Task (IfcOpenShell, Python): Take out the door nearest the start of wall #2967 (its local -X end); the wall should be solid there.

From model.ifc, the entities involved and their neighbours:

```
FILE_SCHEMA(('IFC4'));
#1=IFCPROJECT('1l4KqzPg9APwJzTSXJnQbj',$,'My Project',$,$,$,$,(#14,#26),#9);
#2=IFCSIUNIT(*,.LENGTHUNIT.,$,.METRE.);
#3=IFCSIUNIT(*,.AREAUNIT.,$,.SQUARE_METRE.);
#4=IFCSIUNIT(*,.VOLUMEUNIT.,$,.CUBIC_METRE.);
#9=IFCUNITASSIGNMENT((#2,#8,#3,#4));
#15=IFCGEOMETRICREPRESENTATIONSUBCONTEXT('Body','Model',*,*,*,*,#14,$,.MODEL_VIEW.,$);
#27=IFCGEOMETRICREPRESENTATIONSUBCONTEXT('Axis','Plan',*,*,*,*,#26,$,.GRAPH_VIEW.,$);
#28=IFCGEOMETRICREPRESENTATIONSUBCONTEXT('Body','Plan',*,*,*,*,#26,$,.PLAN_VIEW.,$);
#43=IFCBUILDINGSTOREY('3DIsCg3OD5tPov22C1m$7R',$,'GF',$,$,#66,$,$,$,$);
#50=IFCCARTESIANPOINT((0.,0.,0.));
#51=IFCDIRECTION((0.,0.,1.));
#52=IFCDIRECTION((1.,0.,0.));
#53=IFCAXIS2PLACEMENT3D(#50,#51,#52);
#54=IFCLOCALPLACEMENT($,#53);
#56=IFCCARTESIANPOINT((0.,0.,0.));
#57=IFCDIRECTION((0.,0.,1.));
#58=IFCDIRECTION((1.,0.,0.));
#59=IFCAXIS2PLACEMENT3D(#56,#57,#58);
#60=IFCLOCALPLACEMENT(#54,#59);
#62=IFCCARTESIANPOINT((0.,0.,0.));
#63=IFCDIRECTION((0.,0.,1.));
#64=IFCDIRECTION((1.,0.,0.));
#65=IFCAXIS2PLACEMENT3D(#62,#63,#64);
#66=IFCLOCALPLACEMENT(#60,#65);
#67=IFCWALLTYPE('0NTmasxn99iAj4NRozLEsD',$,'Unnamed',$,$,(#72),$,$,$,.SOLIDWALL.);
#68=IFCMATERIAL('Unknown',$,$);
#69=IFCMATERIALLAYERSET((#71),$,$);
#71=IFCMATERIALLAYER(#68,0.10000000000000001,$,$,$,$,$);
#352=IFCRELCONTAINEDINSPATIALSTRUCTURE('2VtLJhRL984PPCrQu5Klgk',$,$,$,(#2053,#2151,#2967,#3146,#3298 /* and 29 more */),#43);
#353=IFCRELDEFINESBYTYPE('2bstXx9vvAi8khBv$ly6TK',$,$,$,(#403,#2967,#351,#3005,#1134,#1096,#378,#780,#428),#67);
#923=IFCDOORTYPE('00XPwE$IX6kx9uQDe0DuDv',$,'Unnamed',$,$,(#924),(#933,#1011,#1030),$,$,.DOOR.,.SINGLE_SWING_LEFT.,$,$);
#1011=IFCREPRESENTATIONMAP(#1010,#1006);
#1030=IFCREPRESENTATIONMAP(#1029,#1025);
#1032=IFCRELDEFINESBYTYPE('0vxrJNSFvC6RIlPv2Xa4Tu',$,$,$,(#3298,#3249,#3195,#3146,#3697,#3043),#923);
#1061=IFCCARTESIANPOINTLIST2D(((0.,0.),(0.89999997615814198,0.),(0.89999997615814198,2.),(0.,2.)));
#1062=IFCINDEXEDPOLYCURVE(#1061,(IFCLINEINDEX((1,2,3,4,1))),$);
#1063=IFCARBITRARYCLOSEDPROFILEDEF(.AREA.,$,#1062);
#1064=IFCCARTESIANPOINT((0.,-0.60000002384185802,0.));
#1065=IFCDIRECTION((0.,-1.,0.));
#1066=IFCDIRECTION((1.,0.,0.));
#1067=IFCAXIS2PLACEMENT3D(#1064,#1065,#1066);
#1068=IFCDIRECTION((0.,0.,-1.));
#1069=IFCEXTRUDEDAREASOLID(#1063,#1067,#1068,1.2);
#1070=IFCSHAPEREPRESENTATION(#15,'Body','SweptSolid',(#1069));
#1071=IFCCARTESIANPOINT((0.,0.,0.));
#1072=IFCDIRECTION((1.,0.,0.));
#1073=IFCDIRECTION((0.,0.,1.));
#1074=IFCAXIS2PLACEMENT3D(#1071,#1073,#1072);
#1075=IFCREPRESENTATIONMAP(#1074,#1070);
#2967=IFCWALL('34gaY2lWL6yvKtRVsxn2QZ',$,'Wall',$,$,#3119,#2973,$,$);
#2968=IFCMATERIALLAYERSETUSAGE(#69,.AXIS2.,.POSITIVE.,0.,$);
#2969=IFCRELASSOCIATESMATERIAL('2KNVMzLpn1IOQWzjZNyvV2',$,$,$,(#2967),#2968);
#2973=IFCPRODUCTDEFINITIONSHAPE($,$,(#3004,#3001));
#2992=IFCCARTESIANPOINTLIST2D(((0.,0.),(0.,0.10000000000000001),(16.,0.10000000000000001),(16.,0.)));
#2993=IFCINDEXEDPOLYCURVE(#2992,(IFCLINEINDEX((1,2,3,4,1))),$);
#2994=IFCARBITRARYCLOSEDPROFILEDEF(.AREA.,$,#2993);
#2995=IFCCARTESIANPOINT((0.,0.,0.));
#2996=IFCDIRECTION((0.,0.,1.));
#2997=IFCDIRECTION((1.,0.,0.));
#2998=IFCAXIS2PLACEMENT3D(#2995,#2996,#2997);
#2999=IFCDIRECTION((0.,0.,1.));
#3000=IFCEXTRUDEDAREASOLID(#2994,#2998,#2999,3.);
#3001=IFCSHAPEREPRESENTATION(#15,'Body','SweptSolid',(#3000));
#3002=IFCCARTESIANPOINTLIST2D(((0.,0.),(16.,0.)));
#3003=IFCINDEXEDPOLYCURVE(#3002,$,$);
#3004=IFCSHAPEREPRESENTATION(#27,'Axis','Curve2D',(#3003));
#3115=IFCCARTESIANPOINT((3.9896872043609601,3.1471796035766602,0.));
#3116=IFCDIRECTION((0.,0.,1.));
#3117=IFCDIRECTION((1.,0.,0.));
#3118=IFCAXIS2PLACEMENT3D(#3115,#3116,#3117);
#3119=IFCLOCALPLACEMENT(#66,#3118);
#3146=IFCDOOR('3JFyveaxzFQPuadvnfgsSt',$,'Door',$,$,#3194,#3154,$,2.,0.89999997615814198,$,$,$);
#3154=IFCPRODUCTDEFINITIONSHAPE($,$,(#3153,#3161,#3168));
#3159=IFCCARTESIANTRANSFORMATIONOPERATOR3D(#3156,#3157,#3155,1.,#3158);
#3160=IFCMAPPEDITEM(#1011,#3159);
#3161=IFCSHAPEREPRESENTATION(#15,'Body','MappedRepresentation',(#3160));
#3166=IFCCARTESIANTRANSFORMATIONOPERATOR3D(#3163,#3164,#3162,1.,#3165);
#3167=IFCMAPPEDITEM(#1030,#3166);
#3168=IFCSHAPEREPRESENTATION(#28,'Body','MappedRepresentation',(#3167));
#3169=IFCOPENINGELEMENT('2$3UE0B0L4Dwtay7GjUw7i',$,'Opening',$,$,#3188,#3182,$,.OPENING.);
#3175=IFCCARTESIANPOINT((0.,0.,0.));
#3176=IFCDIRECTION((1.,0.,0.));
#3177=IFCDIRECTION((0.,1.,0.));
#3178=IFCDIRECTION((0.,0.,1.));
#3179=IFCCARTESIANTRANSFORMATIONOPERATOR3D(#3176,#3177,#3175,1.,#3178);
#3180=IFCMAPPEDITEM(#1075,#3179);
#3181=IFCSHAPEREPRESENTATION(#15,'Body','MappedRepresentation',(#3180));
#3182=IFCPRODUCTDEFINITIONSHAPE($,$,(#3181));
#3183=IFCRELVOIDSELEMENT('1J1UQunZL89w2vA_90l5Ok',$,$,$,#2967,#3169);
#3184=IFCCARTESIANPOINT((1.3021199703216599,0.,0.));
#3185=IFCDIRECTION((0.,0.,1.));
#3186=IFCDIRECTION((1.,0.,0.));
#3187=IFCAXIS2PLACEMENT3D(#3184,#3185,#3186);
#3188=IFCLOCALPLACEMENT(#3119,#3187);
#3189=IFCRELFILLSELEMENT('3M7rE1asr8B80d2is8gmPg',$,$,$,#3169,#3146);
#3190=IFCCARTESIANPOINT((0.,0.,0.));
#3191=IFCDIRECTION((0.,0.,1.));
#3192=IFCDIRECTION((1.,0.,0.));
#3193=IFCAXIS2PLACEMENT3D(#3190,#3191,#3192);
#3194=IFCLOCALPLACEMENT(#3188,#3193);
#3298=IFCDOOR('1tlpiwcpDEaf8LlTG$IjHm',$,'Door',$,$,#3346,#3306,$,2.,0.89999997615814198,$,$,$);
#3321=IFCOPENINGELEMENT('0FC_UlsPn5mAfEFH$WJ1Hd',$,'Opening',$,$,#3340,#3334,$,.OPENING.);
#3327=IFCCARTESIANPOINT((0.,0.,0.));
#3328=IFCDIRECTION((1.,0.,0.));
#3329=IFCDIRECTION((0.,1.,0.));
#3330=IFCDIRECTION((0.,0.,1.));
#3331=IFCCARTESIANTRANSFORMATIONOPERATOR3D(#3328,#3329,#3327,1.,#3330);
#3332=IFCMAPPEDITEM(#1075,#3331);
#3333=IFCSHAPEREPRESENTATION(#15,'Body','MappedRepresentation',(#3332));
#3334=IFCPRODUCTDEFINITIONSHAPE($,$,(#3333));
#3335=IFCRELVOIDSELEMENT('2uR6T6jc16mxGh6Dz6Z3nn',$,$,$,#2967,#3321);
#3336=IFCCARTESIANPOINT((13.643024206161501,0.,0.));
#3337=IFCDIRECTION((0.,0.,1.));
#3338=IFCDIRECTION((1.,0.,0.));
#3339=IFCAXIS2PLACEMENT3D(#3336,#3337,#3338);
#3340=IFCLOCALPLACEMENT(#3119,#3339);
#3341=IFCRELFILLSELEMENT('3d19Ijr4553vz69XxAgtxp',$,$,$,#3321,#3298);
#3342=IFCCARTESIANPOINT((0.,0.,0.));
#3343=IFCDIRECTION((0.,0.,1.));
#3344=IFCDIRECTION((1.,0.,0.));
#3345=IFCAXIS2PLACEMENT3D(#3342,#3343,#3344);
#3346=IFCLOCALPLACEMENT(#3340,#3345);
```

```python
import ifcopenshell
import ifcopenshell.api.feature
import ifcopenshell.api.root
import ifcopenshell.geom
import ifcopenshell.util.shape

model = ifcopenshell.open("model.ifc")
settings = ifcopenshell.geom.settings()


def volume(element):
    """Net volume in cubic metres, openings subtracted."""
    shape = ifcopenshell.geom.create_shape(settings, element)
    return ifcopenshell.util.shape.get_volume(shape.geometry)


door = model.by_guid("3JFyveaxzFQPuadvnfgsSt")
opening = door.FillsVoids[0].RelatingOpeningElement
wall = opening.VoidsElements[0].RelatingBuildingElement
before = volume(wall)

ifcopenshell.api.root.remove_product(model, product=door)
ifcopenshell.api.feature.remove_feature(model, feature=opening)

after = volume(wall)

print(f"wall volume {before:.3f} -> {after:.3f} m3")

model.write("model_v2.ifc")
```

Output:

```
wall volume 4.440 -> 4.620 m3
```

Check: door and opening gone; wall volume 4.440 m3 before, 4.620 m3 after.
